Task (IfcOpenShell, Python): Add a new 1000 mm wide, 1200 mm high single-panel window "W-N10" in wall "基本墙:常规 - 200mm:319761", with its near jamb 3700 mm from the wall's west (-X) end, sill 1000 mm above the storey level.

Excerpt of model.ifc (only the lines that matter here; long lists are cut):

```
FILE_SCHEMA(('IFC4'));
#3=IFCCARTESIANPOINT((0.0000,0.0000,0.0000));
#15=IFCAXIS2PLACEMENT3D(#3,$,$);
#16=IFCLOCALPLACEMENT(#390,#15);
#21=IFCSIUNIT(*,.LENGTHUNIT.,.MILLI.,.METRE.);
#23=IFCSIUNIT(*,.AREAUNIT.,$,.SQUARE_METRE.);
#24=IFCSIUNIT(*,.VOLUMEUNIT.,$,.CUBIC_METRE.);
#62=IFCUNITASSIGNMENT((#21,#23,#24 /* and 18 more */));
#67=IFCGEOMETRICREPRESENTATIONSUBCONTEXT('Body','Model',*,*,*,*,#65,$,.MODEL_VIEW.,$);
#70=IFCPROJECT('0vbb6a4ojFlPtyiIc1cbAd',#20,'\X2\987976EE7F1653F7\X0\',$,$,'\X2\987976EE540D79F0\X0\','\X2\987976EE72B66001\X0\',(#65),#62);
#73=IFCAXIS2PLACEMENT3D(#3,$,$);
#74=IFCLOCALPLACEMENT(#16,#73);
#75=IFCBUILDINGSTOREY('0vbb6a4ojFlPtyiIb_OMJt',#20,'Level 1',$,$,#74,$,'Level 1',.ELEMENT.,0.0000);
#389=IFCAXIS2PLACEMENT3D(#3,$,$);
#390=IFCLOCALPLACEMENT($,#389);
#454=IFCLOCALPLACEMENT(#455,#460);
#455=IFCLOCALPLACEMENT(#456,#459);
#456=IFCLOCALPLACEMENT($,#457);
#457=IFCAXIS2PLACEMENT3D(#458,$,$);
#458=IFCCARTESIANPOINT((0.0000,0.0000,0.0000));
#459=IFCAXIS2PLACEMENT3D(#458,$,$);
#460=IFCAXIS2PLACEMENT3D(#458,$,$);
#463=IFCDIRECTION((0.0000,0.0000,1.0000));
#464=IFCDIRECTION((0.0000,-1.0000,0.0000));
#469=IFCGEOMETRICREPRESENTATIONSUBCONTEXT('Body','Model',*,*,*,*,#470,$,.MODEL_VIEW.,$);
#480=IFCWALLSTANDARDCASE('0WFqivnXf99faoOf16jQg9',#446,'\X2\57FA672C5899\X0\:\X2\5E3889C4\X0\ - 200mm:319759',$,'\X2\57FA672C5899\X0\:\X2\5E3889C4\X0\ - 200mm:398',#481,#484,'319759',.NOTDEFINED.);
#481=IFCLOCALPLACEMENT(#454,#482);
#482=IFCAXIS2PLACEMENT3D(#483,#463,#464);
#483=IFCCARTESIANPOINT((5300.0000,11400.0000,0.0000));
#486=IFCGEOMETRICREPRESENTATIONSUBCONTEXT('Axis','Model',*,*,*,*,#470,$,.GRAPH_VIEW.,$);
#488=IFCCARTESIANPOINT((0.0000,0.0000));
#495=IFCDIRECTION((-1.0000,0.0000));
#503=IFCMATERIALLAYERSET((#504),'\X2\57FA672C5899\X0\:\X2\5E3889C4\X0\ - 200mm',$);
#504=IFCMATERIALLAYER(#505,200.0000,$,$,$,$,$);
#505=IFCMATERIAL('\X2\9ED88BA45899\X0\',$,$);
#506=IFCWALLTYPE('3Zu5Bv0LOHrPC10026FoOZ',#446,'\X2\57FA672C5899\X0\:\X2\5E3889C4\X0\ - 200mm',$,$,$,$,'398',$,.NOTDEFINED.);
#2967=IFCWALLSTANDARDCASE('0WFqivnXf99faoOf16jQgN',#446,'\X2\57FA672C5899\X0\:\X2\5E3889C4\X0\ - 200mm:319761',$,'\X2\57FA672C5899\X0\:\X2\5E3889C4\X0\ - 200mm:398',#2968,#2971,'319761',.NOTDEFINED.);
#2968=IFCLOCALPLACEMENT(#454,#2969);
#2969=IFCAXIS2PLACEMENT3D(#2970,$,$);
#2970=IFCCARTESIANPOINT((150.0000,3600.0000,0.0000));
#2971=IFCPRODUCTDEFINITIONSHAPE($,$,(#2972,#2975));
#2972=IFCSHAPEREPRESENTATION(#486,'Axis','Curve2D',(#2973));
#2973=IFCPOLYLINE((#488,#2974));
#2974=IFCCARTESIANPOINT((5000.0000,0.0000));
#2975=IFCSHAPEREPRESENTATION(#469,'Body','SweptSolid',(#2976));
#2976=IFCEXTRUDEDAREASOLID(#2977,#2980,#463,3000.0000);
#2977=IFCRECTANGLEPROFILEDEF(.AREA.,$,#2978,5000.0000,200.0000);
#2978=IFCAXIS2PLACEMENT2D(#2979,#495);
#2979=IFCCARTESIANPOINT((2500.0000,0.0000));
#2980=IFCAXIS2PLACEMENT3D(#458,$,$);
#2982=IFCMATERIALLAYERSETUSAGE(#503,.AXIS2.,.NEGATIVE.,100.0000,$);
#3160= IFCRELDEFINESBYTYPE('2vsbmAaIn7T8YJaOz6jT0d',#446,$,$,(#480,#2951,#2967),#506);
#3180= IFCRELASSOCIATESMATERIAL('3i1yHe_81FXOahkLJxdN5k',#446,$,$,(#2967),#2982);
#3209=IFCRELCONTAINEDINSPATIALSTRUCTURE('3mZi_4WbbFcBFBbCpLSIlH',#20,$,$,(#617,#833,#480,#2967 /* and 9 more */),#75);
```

```python
import numpy as np
import ifcopenshell
import ifcopenshell.api.feature
import ifcopenshell.api.geometry
import ifcopenshell.api.root
import ifcopenshell.api.spatial
import ifcopenshell.geom
import ifcopenshell.util.element
import ifcopenshell.util.placement
import ifcopenshell.util.representation
import ifcopenshell.util.shape
import ifcopenshell.util.unit

model = ifcopenshell.open("model.ifc")
unit_scale = ifcopenshell.util.unit.calculate_unit_scale(model)
settings = ifcopenshell.geom.settings()


def volume(element):
    """Net volume in cubic metres, openings subtracted."""
    shape = ifcopenshell.geom.create_shape(settings, element)
    return ifcopenshell.util.shape.get_volume(shape.geometry)


wall = model.by_id(2967)
storey = ifcopenshell.util.element.get_container(wall, ifc_class="IfcBuildingStorey")
context = ifcopenshell.util.representation.get_context(model, "Model", "Body", "MODEL_VIEW")
before = volume(wall)

width, height, from_end, sill = 1, 1.2, 3.7, 1  # metres

# The wall runs along its own X axis, and the end named is its -X end.
wall_shape = ifcopenshell.geom.create_shape(settings, wall)
x, y, z = ifcopenshell.util.shape.get_vertices(wall_shape.geometry).T
start = x.min() + from_end
face, thickness = float(y.min()), float(y.max() - y.min())
wall_matrix = ifcopenshell.util.placement.get_local_placement(wall.ObjectPlacement)
level = ifcopenshell.util.placement.get_local_placement(storey.ObjectPlacement)[2, 3]


def in_wall(x, y):
    """Placement at x, y metres in the wall's axes, at sill height."""
    matrix = wall_matrix.copy()
    matrix[:, 3] = wall_matrix @ np.array([x / unit_scale, y / unit_scale, 0.0, 1.0])
    matrix[2, 3] = level + sill / unit_scale
    return matrix


# Opening: a box that overshoots both wall faces by 50 mm.
opening = ifcopenshell.api.root.create_entity(model, ifc_class="IfcOpeningElement", predefined_type="OPENING")
box = ifcopenshell.api.geometry.add_wall_representation(
    model, context=context, length=width, height=height, thickness=thickness + 0.1
)
ifcopenshell.api.geometry.assign_representation(model, product=opening, representation=box)
ifcopenshell.api.geometry.edit_object_placement(model, product=opening, matrix=in_wall(start, face - 0.05), is_si=False)
ifcopenshell.api.feature.add_feature(model, feature=opening, element=wall)

window = ifcopenshell.api.root.create_entity(model, ifc_class="IfcWindow", name="W-N10", predefined_type="WINDOW")
window.OverallWidth, window.OverallHeight = width / unit_scale, height / unit_scale
window.PartitioningType = "SINGLE_PANEL"
body = ifcopenshell.api.geometry.add_window_representation(
    model,
    context=context,
    overall_width=window.OverallWidth,
    overall_height=window.OverallHeight,
    partition_type="SINGLE_PANEL",
)
ifcopenshell.api.geometry.assign_representation(model, product=window, representation=body)
ifcopenshell.api.spatial.assign_container(model, products=[window], relating_structure=storey)
ifcopenshell.api.feature.add_filling(model, opening=opening, element=window)

# Centre the window in the wall's thickness.
ifcopenshell.api.geometry.edit_object_placement(model, product=window, matrix=in_wall(start, face), is_si=False)
window_shape = ifcopenshell.geom.create_shape(settings, window)
depth = ifcopenshell.util.shape.get_vertices(window_shape.geometry)[:, 1]
offset = face + thickness / 2 - (depth.min() + depth.max()) / 2
ifcopenshell.api.geometry.edit_object_placement(model, product=window, matrix=in_wall(start, offset), is_si=False)

after = volume(wall)

print(f"wall volume {before:.3f} -> {after:.3f} m3")

model.write("model_edited.ifc")
```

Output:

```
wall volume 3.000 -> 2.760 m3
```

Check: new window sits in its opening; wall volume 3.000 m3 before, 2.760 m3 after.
